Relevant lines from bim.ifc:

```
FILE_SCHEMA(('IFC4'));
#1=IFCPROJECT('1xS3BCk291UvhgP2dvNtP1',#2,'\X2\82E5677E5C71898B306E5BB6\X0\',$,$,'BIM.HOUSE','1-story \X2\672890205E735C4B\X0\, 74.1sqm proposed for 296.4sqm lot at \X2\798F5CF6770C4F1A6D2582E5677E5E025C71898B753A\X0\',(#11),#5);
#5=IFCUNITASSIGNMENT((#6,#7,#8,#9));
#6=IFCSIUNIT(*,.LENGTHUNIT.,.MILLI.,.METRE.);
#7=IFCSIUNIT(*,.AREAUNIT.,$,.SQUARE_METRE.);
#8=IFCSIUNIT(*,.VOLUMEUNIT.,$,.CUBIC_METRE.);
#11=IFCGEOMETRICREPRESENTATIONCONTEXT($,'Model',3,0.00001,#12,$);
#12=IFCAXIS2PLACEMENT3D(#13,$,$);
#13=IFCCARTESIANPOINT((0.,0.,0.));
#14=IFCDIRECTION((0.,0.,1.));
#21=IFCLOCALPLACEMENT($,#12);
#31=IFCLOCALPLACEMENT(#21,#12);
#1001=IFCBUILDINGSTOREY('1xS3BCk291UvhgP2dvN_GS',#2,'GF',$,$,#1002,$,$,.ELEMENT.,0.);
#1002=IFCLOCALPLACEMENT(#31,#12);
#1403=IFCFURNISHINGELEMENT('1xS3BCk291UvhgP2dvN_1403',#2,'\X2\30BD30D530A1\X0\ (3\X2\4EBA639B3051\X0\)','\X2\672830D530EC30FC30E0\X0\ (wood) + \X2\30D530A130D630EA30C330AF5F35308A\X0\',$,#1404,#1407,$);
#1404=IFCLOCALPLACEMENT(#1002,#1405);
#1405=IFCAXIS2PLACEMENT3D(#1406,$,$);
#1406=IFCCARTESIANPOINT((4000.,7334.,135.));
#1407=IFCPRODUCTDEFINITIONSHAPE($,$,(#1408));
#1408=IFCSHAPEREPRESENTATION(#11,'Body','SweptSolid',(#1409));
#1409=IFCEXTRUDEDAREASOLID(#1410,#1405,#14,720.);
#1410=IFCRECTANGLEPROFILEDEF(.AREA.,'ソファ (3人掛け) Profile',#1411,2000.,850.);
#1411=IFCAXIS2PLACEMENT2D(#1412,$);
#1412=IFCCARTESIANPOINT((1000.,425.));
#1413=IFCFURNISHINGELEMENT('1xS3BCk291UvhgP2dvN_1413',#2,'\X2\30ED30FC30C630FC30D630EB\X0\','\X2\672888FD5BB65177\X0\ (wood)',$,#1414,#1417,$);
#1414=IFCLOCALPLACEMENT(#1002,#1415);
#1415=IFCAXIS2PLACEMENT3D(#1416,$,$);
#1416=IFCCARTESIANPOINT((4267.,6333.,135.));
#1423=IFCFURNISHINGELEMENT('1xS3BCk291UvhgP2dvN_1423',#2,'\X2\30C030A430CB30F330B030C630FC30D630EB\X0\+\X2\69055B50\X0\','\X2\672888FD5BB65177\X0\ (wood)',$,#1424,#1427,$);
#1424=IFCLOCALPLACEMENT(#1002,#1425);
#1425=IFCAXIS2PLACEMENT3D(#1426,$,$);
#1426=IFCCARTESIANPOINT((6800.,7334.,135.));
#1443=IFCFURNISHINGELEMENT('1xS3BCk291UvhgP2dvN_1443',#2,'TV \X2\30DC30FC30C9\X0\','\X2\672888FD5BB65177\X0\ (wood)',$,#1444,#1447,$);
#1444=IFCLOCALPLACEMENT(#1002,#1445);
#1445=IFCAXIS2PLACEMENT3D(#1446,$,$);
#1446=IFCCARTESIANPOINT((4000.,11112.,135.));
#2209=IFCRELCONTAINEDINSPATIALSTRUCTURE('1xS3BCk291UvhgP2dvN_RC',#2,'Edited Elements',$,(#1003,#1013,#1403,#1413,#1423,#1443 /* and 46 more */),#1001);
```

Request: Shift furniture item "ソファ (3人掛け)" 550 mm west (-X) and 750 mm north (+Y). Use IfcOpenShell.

```python
import ifcopenshell
import ifcopenshell.api.geometry
import ifcopenshell.util.placement
import ifcopenshell.util.unit

model = ifcopenshell.open("bim.ifc")
unit_scale = ifcopenshell.util.unit.calculate_unit_scale(model)

item = model.by_guid("1xS3BCk291UvhgP2dvN_1403")
matrix = ifcopenshell.util.placement.get_local_placement(item.ObjectPlacement)
matrix[0, 3] -= 0.55 / unit_scale
matrix[1, 3] += 0.75 / unit_scale
ifcopenshell.api.geometry.edit_object_placement(model, product=item, matrix=matrix, is_si=False)

print(ifcopenshell.util.placement.get_local_placement(item.ObjectPlacement).round(3) + 0.0)

model.write("bim-out.ifc")
```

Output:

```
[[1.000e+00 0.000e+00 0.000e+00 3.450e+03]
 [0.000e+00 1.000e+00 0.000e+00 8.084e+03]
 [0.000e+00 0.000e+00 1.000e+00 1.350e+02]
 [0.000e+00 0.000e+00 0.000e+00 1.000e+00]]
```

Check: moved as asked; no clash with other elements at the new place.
